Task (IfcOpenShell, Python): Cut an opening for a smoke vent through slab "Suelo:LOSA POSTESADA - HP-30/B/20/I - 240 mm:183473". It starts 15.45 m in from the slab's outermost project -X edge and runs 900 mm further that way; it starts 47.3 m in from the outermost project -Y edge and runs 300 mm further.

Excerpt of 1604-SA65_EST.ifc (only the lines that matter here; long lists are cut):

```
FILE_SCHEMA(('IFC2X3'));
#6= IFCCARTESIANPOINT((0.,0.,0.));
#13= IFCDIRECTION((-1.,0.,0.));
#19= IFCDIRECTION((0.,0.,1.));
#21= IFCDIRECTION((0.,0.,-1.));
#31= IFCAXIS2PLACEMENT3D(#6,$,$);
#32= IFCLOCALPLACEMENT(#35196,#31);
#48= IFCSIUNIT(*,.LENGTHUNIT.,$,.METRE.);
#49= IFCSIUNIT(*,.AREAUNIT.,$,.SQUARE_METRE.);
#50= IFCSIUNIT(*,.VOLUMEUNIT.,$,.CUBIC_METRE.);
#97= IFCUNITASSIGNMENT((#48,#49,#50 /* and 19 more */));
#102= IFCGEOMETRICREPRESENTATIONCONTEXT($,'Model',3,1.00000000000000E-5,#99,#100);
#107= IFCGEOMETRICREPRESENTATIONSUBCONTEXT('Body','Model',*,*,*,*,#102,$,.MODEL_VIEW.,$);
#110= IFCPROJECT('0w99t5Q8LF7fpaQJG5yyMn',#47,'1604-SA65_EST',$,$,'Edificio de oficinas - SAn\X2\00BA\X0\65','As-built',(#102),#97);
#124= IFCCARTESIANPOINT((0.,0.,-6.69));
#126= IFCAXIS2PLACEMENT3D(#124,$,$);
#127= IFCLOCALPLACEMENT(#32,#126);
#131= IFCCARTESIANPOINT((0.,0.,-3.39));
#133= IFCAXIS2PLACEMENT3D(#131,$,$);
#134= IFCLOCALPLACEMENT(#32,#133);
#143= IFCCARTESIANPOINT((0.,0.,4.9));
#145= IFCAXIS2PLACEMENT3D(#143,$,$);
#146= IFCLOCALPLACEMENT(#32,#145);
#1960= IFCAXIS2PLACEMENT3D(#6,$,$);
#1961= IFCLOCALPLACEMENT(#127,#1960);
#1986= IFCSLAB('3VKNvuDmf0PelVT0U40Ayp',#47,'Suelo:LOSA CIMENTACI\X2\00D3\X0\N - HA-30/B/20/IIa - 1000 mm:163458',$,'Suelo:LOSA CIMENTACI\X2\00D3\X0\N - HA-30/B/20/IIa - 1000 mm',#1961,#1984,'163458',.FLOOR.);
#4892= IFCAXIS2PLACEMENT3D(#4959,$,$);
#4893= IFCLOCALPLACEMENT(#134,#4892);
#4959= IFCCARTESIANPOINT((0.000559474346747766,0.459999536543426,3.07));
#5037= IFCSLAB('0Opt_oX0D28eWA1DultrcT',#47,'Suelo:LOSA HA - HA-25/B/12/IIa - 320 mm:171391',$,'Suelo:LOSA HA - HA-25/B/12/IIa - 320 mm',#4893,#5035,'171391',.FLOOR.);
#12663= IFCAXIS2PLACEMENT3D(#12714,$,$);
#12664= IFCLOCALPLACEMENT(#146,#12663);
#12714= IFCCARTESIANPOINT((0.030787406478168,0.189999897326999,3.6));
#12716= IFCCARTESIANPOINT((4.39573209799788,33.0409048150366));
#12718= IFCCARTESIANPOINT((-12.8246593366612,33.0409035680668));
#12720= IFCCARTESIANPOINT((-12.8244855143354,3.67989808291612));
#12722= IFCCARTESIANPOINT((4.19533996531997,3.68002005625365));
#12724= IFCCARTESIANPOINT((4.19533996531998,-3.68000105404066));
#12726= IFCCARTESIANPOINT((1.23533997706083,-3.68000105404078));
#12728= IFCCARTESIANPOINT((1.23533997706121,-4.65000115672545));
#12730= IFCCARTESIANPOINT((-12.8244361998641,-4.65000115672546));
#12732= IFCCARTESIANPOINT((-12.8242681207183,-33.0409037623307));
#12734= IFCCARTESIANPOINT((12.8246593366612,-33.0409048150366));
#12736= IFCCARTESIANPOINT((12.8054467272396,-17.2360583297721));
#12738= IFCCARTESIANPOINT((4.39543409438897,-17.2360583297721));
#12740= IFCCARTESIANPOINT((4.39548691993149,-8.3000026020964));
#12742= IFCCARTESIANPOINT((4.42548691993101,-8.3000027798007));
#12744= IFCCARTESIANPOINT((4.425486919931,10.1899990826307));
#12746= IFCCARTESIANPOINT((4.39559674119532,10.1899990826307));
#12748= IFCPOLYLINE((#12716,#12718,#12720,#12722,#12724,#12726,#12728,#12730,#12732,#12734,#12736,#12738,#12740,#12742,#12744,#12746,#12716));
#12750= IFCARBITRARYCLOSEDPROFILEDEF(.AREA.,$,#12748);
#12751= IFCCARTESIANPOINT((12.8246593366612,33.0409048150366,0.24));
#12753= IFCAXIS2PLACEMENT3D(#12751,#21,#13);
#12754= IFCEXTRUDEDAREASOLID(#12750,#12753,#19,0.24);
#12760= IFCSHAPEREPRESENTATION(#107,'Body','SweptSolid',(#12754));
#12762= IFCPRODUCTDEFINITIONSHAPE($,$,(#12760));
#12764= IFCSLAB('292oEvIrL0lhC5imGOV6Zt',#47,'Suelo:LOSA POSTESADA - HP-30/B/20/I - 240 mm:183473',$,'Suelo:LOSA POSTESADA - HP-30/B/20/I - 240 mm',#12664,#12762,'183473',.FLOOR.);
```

```python
import numpy as np
import ifcopenshell
import ifcopenshell.api.feature
import ifcopenshell.api.geometry
import ifcopenshell.api.root
import ifcopenshell.geom
import ifcopenshell.util.placement
import ifcopenshell.util.representation
import ifcopenshell.util.shape
import ifcopenshell.util.unit

model = ifcopenshell.open("1604-SA65_EST.ifc")
unit_scale = ifcopenshell.util.unit.calculate_unit_scale(model)
settings = ifcopenshell.geom.settings()


def volume(element):
    """Net volume in cubic metres, openings subtracted."""
    shape = ifcopenshell.geom.create_shape(settings, element)
    return ifcopenshell.util.shape.get_volume(shape.geometry)


slab = model.by_guid("292oEvIrL0lhC5imGOV6Zt")
before = volume(slab)

# Extent in the slab's own axes, in metres. The edges named are its -X and -Y sides.
slab_shape = ifcopenshell.geom.create_shape(settings, slab)
vertices = ifcopenshell.util.shape.get_vertices(slab_shape.geometry)
x_min, y_min, bottom = vertices.min(axis=0)
top = vertices[:, 2].max()

opening = ifcopenshell.api.root.create_entity(model, ifc_class="IfcOpeningElement", name="Smoke vent opening")
context = ifcopenshell.util.representation.get_context(model, "Model", "Body", "MODEL_VIEW")
width, depth = 0.9, 0.3
outline = [(0.0, 0.0), (width, 0.0), (width, depth), (0.0, depth), (0.0, 0.0)]
# Overshoot both faces by 50 mm so the cut is clean.
shape = ifcopenshell.api.geometry.add_slab_representation(
    model, context=context, depth=top - bottom + 0.1, polyline=outline
)
ifcopenshell.api.geometry.assign_representation(model, product=opening, representation=shape)

matrix = ifcopenshell.util.placement.get_local_placement(slab.ObjectPlacement)
matrix[:, 3] = matrix @ np.append(np.array([x_min + 15.45, y_min + 47.3, bottom - 0.05]) / unit_scale, 1.0)
ifcopenshell.api.geometry.edit_object_placement(model, product=opening, matrix=matrix, is_si=False)
ifcopenshell.api.feature.add_feature(model, feature=opening, element=slab)

after = volume(slab)

print(f"slab volume {before:.3f} -> {after:.3f} m3")

model.write("1604-SA65_EST_v2.ifc")
```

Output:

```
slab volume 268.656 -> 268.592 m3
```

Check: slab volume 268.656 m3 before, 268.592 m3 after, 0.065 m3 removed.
